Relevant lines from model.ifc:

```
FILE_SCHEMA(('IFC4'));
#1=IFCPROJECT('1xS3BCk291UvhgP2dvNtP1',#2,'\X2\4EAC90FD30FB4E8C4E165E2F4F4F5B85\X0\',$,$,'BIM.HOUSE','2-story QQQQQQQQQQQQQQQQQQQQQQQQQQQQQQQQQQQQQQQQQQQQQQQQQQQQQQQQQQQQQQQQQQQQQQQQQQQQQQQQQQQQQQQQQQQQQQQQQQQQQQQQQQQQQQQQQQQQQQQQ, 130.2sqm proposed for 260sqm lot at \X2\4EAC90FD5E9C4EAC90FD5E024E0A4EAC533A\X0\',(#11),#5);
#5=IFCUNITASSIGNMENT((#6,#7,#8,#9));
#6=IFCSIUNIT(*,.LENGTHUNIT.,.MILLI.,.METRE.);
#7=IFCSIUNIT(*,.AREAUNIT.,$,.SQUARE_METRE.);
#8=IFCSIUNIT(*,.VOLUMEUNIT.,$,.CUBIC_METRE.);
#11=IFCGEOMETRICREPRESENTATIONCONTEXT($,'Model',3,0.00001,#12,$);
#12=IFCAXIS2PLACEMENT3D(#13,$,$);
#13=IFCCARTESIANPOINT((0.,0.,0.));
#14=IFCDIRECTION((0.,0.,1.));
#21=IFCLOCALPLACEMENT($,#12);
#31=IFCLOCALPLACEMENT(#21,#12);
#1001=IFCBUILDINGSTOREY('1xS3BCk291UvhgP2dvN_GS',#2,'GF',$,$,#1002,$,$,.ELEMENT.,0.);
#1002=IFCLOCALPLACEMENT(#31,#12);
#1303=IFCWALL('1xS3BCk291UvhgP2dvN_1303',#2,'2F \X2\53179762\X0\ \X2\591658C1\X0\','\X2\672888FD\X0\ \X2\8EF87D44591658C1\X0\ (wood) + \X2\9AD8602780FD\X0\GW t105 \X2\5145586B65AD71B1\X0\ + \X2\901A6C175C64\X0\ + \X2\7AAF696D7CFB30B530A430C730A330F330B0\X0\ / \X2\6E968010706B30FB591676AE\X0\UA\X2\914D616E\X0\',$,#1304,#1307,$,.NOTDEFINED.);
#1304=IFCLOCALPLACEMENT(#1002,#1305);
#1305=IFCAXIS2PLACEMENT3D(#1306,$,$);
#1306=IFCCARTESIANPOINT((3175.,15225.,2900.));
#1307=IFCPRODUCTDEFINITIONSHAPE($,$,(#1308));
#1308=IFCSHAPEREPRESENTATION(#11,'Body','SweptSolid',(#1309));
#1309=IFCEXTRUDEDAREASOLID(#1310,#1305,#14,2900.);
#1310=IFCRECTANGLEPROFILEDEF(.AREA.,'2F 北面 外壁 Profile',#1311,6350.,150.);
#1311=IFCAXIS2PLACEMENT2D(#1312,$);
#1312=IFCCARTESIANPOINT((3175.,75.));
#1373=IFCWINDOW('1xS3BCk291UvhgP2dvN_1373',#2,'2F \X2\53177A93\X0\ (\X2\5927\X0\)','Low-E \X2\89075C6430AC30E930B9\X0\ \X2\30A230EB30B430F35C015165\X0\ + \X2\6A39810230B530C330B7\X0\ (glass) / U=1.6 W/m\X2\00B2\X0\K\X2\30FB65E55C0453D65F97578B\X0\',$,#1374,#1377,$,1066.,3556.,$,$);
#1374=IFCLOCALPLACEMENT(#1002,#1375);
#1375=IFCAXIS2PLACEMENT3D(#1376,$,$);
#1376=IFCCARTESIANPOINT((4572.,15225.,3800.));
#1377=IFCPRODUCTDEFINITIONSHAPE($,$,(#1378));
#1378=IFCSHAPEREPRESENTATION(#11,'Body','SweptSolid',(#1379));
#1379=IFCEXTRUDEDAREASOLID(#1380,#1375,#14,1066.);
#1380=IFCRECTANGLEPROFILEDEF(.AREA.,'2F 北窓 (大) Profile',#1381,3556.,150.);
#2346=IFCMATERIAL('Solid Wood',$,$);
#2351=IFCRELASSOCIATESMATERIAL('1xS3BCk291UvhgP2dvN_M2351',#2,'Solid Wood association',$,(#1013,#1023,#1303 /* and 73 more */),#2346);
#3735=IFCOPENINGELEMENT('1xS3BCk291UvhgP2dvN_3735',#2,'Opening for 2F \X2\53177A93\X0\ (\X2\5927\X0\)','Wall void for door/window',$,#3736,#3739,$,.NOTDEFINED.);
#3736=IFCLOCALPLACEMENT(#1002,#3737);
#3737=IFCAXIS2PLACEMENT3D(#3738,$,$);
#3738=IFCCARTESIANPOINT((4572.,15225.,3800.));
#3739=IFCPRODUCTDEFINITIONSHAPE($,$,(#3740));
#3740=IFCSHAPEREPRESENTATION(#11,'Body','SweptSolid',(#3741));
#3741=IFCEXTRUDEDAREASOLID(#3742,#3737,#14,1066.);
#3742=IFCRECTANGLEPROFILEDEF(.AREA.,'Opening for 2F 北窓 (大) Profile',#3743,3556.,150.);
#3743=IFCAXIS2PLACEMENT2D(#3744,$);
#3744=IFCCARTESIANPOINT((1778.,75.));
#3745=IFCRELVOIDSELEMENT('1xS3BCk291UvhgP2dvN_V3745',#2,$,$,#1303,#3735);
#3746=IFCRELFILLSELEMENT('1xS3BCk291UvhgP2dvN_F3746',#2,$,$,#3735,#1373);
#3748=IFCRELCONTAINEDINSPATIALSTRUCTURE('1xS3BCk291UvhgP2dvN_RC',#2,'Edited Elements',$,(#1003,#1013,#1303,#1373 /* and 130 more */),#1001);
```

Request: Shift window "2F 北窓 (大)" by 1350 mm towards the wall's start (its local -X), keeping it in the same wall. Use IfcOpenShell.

```python
import ifcopenshell
import ifcopenshell.api.geometry
import ifcopenshell.util.placement

model = ifcopenshell.open("model.ifc")

window = model.by_guid("1xS3BCk291UvhgP2dvN_1373")
opening = window.FillsVoids[0].RelatingOpeningElement
wall = opening.VoidsElements[0].RelatingBuildingElement

wall_matrix = ifcopenshell.util.placement.get_local_placement(wall.ObjectPlacement)
shift = wall_matrix[:3, 0] * -1350.0
before = ifcopenshell.util.placement.get_local_placement(window.ObjectPlacement)[:3, 3].copy()

# The window is not placed relative to its opening, so move both.
for product in (opening, window):
    matrix = ifcopenshell.util.placement.get_local_placement(product.ObjectPlacement)
    matrix[:3, 3] += shift
    ifcopenshell.api.geometry.edit_object_placement(model, product=product, matrix=matrix, is_si=False)

after = ifcopenshell.util.placement.get_local_placement(window.ObjectPlacement)[:3, 3]
print("window moved by", (after - before).round(3) + 0.0)

model.write("model_rev.ifc")
```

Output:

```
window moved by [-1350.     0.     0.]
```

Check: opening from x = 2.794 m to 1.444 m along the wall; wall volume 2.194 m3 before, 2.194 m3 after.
